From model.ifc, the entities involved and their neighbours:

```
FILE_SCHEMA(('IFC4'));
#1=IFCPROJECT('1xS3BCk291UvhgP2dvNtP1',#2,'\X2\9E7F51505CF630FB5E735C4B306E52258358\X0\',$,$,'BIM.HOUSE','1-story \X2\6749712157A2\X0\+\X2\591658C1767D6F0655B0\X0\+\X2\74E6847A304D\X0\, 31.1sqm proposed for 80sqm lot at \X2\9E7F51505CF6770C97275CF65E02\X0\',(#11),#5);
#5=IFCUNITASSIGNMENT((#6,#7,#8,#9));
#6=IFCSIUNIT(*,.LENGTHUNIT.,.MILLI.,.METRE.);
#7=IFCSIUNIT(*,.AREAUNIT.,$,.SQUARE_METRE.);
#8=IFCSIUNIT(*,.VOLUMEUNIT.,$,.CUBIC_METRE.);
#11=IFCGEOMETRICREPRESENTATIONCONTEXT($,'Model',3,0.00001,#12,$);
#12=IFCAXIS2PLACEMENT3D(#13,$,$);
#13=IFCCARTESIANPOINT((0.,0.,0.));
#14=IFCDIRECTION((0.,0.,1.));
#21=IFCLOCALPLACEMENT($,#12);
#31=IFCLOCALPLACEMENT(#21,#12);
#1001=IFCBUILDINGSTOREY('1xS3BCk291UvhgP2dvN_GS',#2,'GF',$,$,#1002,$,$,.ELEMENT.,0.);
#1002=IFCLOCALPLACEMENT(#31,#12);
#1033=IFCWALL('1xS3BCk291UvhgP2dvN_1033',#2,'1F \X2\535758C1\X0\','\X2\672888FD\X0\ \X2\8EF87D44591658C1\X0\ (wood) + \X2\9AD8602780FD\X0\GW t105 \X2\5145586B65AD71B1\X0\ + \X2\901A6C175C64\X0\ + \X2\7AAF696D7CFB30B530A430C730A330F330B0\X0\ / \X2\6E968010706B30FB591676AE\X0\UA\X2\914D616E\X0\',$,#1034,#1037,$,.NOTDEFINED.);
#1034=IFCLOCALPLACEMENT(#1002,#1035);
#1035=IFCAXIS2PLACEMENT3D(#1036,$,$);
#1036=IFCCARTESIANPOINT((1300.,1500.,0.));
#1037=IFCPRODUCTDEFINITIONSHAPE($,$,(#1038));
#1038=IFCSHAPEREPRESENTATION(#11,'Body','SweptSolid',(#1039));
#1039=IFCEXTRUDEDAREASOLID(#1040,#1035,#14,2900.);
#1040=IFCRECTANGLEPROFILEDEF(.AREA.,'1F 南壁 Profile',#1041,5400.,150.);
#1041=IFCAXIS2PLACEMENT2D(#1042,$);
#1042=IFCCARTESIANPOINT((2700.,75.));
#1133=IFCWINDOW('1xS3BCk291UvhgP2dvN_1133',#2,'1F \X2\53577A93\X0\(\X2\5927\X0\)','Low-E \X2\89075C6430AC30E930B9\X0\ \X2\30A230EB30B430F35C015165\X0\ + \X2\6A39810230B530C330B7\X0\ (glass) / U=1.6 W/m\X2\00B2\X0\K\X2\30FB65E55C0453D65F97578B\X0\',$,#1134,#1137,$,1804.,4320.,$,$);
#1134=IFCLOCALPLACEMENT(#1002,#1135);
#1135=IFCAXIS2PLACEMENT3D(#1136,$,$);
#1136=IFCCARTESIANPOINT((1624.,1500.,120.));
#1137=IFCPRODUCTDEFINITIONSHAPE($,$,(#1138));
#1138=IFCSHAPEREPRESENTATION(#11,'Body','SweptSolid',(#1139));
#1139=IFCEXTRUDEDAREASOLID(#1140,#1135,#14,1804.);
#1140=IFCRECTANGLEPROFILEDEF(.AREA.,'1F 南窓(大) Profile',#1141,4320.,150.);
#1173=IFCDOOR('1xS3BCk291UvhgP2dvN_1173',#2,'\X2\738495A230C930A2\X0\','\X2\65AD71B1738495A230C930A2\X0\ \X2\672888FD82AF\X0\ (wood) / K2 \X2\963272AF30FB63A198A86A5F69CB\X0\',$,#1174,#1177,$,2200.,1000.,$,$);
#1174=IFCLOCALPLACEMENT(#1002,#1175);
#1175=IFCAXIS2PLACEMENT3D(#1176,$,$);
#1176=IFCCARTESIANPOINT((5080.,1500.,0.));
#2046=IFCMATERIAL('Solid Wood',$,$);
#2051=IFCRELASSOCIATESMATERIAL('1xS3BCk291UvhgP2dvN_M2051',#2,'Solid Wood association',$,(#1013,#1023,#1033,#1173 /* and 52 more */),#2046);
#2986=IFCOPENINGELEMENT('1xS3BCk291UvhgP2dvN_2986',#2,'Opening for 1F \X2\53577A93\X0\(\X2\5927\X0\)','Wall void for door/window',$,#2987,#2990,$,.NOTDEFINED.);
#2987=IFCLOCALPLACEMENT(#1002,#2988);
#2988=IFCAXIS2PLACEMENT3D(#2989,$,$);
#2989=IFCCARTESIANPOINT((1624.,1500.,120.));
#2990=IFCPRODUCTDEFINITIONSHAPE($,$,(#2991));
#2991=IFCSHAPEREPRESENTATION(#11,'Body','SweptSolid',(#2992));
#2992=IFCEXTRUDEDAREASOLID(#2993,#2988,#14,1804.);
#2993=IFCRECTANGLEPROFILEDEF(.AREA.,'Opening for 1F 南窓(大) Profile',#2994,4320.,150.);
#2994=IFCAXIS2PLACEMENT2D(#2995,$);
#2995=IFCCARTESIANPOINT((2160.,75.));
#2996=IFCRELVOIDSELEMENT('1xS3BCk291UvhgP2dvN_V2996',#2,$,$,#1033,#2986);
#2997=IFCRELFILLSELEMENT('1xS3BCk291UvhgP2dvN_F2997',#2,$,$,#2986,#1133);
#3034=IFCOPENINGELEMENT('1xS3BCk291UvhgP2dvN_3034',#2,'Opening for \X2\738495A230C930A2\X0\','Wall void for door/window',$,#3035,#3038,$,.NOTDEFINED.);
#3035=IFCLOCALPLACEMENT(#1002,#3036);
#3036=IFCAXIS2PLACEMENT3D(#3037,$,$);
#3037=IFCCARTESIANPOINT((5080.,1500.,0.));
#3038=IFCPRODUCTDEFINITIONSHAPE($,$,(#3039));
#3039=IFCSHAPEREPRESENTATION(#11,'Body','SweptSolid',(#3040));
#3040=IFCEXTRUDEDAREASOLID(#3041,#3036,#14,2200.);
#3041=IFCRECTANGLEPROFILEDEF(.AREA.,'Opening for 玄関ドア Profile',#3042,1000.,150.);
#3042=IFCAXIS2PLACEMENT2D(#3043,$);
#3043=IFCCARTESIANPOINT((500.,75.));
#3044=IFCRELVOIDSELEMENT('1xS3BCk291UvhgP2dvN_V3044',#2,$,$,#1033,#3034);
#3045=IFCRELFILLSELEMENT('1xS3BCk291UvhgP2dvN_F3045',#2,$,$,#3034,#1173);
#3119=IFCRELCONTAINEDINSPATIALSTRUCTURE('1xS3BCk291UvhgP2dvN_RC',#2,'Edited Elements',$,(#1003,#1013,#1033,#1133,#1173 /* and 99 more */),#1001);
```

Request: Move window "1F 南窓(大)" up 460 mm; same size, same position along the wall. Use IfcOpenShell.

```python
import numpy as np
import ifcopenshell
import ifcopenshell.api.geometry
import ifcopenshell.util.placement
import ifcopenshell.util.unit

model = ifcopenshell.open("model.ifc")
unit_scale = ifcopenshell.util.unit.calculate_unit_scale(model)

window = model.by_guid("1xS3BCk291UvhgP2dvN_1133")
opening = window.FillsVoids[0].RelatingOpeningElement
dz = 0.46 / unit_scale

shift = np.array([0.0, 0.0, dz])
# The window is not placed relative to its opening, so move both.
for product in (opening, window):
    matrix = ifcopenshell.util.placement.get_local_placement(product.ObjectPlacement)
    matrix[:3, 3] += shift
    ifcopenshell.api.geometry.edit_object_placement(model, product=product, matrix=matrix, is_si=False)

print(f"moved by {dz * unit_scale:+.3f} m")

model.write("model_rev.ifc")
```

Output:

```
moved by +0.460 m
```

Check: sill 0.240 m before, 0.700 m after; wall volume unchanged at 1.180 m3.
